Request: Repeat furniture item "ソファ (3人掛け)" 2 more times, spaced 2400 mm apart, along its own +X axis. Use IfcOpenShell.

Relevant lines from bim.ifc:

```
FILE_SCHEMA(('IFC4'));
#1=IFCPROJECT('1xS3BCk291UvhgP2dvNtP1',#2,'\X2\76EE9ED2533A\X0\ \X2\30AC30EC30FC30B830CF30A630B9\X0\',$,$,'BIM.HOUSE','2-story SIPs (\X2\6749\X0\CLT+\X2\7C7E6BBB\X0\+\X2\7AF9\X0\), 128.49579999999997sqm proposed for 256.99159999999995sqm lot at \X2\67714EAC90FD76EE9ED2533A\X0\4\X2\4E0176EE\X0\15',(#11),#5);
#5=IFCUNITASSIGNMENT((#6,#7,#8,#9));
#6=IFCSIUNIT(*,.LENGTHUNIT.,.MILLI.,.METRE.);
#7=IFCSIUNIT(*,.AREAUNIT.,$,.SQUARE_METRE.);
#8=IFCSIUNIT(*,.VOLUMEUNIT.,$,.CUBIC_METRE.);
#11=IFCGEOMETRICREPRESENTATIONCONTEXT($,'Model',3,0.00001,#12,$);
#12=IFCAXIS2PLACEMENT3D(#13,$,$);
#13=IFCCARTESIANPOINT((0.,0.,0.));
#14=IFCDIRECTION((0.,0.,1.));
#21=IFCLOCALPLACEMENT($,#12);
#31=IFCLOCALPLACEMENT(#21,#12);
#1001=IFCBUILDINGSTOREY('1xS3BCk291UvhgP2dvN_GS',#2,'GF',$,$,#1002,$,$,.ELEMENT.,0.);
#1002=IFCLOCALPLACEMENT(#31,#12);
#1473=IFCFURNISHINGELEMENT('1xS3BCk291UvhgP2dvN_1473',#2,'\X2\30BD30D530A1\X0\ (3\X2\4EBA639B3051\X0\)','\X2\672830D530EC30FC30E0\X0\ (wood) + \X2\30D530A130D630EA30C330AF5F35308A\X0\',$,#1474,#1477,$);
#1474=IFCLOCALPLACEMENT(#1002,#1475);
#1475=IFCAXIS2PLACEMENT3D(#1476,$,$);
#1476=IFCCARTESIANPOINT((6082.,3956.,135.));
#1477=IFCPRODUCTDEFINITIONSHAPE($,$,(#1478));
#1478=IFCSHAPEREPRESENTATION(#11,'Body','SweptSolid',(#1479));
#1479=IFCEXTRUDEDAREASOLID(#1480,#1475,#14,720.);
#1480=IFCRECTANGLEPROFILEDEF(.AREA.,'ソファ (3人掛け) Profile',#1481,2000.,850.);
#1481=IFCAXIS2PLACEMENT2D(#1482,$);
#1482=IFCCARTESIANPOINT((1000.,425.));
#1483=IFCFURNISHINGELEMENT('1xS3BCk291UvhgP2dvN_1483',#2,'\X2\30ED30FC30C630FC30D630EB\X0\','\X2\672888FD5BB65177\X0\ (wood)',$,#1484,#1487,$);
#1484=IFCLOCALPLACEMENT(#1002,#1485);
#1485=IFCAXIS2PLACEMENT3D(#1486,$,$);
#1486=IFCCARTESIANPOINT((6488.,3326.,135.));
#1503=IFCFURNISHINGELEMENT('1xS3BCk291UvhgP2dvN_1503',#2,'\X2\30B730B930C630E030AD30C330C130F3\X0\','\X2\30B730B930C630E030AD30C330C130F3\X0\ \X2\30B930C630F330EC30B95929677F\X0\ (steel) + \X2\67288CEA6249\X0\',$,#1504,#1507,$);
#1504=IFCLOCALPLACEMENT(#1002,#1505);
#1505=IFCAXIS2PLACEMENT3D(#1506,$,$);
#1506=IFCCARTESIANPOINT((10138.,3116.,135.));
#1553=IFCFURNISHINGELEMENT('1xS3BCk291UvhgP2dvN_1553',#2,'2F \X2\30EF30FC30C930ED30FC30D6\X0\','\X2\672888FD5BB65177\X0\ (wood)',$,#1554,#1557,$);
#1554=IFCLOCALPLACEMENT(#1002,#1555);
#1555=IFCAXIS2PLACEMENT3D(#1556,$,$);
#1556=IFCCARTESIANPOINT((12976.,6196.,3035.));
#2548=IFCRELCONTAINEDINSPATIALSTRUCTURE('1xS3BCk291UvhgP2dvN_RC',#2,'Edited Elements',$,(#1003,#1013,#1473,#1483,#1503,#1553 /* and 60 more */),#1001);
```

```python
import ifcopenshell
import ifcopenshell.api.geometry
import ifcopenshell.api.root
import ifcopenshell.util.element
import ifcopenshell.util.placement

model = ifcopenshell.open("bim.ifc")


def reuse_history(source, copy):
    """copy_class also copies each property set's owner history, people and application; keep the originals."""
    for rel in copy.IsDefinedBy:
        if rel.is_a("IfcRelDefinesByProperties") and (history := rel.RelatingPropertyDefinition.OwnerHistory):
            rel.RelatingPropertyDefinition.OwnerHistory = source.OwnerHistory
            ifcopenshell.util.element.remove_deep2(model, history)


source = model.by_guid("1xS3BCk291UvhgP2dvN_1473")
base = ifcopenshell.util.placement.get_local_placement(source.ObjectPlacement)
step = base[:3, 0] * 2400.0

for i in range(1, 3):
    copy = ifcopenshell.api.root.copy_class(model, product=source)
    copy.Representation = ifcopenshell.util.element.copy_deep(
        model, source.Representation, exclude=["IfcGeometricRepresentationContext", "IfcRepresentationMap"]
    )
    reuse_history(source, copy)
    matrix = base.copy()
    matrix[:3, 3] += i * step
    print("added at", matrix[:3, 3].round(3) + 0.0)
    ifcopenshell.api.geometry.edit_object_placement(model, product=copy, matrix=matrix, is_si=False)

model.write("bim_v2.ifc")
```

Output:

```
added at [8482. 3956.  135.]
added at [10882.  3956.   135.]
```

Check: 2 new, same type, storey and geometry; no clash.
